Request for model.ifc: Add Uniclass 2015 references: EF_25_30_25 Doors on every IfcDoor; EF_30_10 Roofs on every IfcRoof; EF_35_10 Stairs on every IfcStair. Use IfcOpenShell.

First a look at what the model holds.

```python
import ifcopenshell

model = ifcopenshell.open("model.ifc")
print(model.schema)
print("classifications:", [c.Name for c in model.by_type("IfcClassification")])
for ifc_class in ("IfcDoor", "IfcRoof", "IfcStair", "IfcWall", "IfcWindow"):
    print(ifc_class, len(model.by_type(ifc_class)))
```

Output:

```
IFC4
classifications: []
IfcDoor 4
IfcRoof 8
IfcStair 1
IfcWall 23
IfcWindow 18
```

```python
import ifcopenshell
import ifcopenshell.api.classification

model = ifcopenshell.open("model.ifc")

system = ifcopenshell.api.classification.add_classification(model, classification="Uniclass 2015")

codes = {
    "IfcDoor": ("EF_25_30_25", "Doors"),
    "IfcRoof": ("EF_30_10", "Roofs"),
    "IfcStair": ("EF_35_10", "Stairs"),
}
for ifc_class, (code, name) in codes.items():
    products = model.by_type(ifc_class)
    ifcopenshell.api.classification.add_reference(
        model, products=products, classification=system, identification=code, name=name
    )
    print(code, len(products))

model.write("model-out.ifc")
```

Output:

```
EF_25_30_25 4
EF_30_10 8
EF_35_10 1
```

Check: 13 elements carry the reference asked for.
